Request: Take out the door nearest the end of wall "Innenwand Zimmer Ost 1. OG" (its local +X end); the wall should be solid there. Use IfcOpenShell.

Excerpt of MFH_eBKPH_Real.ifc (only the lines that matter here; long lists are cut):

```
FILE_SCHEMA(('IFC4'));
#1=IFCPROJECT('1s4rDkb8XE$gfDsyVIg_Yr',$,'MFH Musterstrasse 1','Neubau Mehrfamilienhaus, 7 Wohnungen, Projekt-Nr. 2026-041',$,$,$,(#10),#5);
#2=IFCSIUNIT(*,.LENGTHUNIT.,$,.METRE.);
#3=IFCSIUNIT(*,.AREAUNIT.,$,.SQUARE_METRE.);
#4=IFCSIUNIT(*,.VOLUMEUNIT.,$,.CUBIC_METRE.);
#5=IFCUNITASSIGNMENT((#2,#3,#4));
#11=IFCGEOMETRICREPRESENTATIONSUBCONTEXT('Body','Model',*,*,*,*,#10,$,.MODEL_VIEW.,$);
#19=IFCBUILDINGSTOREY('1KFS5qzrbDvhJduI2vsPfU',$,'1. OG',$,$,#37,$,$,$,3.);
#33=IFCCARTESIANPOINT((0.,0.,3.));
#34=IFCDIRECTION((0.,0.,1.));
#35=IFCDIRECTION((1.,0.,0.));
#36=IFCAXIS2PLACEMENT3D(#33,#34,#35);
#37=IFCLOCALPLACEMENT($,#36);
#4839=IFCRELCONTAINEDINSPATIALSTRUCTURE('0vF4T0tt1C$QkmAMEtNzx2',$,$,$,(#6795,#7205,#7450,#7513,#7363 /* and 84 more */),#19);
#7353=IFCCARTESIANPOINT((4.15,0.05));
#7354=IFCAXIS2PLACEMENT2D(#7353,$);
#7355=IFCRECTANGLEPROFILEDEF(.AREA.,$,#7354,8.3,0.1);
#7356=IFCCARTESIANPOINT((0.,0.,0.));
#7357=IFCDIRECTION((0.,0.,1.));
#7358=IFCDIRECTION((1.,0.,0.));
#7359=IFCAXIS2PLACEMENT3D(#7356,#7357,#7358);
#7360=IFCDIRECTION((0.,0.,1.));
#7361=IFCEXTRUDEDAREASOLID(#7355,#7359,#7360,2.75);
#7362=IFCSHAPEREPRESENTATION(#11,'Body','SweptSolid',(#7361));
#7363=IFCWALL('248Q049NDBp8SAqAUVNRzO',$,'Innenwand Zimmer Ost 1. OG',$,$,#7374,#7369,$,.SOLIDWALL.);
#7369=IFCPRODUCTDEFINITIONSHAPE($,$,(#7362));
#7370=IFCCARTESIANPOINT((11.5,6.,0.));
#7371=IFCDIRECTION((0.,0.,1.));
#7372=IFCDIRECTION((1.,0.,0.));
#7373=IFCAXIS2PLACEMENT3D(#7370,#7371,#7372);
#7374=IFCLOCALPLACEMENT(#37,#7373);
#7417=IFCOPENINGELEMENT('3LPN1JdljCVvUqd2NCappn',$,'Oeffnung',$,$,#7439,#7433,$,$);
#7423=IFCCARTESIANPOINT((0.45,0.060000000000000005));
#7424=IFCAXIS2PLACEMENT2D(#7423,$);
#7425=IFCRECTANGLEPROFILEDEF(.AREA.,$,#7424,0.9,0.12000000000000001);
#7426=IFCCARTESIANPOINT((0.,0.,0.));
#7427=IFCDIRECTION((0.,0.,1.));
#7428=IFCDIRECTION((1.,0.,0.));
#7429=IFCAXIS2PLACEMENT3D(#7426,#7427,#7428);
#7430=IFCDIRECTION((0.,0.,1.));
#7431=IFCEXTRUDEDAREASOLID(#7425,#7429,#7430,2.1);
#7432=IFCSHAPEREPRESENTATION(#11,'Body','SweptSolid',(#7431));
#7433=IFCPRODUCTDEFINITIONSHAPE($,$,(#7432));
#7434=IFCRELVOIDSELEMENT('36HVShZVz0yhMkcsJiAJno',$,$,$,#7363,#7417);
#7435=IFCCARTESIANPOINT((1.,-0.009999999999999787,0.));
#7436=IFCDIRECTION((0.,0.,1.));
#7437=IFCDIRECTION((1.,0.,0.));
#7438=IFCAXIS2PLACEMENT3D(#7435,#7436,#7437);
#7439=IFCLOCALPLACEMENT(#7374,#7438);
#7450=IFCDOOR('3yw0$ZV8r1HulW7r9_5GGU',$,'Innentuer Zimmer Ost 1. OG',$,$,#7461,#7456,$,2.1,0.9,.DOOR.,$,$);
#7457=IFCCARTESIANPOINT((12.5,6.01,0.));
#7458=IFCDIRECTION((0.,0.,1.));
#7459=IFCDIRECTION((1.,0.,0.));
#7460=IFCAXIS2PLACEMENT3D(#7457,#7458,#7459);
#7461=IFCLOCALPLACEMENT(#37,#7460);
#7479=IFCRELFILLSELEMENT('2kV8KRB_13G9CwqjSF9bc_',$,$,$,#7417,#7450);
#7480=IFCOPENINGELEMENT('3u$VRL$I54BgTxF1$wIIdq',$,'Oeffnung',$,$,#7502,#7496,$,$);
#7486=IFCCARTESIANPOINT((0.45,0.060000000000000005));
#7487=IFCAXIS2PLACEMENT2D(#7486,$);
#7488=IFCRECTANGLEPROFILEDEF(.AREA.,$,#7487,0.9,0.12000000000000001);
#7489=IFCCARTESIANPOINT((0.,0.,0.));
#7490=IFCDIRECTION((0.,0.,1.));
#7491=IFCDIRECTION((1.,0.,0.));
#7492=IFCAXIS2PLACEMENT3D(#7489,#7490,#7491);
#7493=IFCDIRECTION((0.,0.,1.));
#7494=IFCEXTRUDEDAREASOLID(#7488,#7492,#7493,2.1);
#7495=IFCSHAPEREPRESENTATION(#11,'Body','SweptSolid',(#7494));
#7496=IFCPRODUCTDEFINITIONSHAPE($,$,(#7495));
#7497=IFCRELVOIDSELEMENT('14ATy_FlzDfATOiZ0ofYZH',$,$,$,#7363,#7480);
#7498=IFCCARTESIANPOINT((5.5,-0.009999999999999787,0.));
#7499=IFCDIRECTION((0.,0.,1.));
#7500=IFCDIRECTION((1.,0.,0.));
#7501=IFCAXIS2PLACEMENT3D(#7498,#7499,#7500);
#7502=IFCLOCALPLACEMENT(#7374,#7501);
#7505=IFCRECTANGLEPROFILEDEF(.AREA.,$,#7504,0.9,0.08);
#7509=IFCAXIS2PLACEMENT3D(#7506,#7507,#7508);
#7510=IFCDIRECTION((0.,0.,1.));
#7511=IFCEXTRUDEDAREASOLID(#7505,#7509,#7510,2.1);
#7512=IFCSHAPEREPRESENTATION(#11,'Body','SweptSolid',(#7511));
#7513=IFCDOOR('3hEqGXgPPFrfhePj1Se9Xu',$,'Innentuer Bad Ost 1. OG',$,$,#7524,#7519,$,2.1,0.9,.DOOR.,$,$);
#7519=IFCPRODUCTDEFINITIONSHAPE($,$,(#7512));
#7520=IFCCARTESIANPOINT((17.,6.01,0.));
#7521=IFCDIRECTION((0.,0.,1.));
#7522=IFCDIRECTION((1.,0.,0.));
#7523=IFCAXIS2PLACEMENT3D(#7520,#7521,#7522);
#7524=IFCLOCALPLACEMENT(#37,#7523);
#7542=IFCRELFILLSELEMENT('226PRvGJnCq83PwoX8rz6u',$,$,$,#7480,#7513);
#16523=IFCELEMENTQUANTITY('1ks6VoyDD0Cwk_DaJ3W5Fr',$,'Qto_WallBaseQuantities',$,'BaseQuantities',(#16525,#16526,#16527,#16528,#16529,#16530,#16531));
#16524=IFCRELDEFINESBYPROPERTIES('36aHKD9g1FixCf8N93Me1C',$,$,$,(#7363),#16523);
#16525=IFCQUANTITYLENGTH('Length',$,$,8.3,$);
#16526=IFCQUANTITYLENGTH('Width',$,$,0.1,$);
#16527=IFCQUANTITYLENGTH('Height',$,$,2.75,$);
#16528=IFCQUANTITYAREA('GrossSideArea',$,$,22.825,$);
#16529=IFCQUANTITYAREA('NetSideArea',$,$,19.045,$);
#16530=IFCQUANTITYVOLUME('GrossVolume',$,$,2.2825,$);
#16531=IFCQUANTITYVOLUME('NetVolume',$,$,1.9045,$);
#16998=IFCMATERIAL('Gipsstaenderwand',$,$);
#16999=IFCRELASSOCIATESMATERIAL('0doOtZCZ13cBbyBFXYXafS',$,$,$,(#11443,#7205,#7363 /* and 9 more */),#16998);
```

```python
import ifcopenshell
import ifcopenshell.api.feature
import ifcopenshell.api.pset
import ifcopenshell.api.root
import ifcopenshell.geom
import ifcopenshell.util.element
import ifcopenshell.util.shape
import ifcopenshell.util.unit

model = ifcopenshell.open("MFH_eBKPH_Real.ifc")
area_scale = ifcopenshell.util.unit.calculate_unit_scale(model, "AREAUNIT")
volume_scale = ifcopenshell.util.unit.calculate_unit_scale(model, "VOLUMEUNIT")
settings = ifcopenshell.geom.settings()


def volume(element):
    """Net volume in cubic metres, openings subtracted."""
    shape = ifcopenshell.geom.create_shape(settings, element)
    return ifcopenshell.util.shape.get_volume(shape.geometry)


door = model.by_guid("3hEqGXgPPFrfhePj1Se9Xu")
opening = door.FillsVoids[0].RelatingOpeningElement
wall = opening.VoidsElements[0].RelatingBuildingElement
before = volume(wall)

ifcopenshell.api.root.remove_product(model, product=door)
ifcopenshell.api.feature.remove_feature(model, feature=opening)

after = volume(wall)
thickness = 0.1  # wall thickness in metres

# Update the wall's stored quantities.
qto = model.by_id(ifcopenshell.util.element.get_pset(wall, "Qto_WallBaseQuantities", should_inherit=False)["id"])
ifcopenshell.api.pset.edit_qto(model, qto=qto, properties={
    "NetSideArea": after / thickness / area_scale,
    "NetVolume": after / volume_scale,
})

print(f"wall volume {before:.3f} -> {after:.3f} m3")

model.write("MFH_eBKPH_Real_v2.ifc")
```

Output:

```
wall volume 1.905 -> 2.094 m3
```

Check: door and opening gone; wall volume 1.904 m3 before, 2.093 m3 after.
